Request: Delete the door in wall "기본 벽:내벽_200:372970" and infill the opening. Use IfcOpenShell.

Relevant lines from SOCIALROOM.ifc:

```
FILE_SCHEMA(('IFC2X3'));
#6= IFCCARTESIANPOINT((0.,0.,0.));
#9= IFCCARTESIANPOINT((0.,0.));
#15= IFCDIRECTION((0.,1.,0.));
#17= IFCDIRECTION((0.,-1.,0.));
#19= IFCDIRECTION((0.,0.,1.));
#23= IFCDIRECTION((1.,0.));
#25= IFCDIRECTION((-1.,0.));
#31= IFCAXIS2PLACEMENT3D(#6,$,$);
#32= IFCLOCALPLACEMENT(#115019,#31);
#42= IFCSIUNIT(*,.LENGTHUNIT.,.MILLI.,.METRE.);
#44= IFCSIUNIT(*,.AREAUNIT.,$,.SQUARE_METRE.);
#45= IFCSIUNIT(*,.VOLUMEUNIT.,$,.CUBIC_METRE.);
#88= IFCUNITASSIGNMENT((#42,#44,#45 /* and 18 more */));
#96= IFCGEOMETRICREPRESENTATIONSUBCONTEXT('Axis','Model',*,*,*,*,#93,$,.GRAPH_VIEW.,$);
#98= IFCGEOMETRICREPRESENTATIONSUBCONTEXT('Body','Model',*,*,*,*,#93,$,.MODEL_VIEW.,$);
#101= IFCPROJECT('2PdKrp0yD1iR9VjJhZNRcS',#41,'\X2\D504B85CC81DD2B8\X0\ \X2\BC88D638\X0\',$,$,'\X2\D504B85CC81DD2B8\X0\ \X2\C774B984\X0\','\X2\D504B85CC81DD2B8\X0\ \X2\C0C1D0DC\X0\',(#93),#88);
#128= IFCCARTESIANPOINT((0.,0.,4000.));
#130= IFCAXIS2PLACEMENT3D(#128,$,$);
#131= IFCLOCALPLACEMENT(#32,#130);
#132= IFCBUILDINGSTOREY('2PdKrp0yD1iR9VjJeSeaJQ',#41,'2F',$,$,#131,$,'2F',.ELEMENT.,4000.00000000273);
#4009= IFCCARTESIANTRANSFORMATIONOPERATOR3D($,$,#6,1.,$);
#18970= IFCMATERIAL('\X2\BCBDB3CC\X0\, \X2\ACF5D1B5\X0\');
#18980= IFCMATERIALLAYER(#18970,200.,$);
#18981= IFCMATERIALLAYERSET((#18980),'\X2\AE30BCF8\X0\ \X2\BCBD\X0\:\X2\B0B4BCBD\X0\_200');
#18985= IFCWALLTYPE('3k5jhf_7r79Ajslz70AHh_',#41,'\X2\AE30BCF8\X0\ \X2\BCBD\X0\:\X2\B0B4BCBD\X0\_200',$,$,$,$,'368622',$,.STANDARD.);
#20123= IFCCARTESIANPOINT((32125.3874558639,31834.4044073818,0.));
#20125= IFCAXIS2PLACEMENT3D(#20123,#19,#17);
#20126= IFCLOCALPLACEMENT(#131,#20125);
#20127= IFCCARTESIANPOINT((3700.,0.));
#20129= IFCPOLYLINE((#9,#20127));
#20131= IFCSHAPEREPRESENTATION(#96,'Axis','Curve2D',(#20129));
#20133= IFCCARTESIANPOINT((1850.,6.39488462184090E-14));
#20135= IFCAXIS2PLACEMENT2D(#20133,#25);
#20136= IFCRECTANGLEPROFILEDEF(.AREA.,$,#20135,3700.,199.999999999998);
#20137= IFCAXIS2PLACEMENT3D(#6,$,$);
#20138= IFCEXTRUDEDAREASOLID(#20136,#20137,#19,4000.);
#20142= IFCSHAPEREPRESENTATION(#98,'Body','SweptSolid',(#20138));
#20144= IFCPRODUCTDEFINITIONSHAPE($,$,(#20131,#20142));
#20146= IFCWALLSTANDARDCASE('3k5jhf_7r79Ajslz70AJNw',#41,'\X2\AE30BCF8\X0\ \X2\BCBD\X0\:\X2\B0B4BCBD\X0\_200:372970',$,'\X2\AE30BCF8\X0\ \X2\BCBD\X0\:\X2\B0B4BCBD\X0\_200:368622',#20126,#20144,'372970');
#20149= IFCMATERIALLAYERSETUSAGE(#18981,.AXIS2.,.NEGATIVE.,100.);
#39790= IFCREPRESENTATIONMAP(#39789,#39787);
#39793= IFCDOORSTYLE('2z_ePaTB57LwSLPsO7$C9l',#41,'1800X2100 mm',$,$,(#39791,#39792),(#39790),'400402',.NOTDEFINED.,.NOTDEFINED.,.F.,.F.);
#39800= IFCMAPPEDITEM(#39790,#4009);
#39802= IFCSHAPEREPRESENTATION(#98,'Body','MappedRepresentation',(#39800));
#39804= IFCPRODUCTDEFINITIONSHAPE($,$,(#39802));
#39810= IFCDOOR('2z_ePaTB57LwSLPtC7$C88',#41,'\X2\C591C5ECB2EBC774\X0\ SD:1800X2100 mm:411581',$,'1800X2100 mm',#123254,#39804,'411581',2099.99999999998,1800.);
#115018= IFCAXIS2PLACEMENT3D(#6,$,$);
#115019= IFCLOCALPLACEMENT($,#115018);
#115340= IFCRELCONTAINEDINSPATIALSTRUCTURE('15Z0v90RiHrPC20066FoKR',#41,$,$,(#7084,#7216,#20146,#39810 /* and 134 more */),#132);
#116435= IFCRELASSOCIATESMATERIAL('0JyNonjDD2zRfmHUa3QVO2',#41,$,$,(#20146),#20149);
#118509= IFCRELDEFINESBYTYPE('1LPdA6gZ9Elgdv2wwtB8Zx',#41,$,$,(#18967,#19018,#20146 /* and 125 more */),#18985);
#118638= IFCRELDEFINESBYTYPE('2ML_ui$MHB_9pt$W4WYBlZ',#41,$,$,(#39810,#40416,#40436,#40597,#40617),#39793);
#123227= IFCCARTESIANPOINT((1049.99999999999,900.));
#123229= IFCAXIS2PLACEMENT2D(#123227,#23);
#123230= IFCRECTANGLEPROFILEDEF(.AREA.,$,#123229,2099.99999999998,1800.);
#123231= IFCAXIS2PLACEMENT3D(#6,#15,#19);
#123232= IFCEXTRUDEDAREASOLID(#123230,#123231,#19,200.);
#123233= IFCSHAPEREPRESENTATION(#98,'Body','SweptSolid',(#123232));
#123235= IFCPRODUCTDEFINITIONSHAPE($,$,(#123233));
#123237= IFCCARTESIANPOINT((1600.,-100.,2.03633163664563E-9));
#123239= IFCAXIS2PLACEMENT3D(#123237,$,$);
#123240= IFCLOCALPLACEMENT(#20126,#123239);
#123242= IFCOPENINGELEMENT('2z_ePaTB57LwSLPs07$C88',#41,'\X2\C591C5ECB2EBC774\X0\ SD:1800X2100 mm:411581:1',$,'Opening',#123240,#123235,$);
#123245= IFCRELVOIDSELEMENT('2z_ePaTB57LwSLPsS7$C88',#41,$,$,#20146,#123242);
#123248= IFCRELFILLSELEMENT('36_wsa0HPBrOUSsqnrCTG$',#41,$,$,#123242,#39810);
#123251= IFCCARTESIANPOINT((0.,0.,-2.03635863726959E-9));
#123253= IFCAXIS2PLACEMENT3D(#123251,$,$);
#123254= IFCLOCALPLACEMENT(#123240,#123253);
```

```python
import ifcopenshell
import ifcopenshell.api.feature
import ifcopenshell.api.root
import ifcopenshell.geom
import ifcopenshell.util.shape

model = ifcopenshell.open("SOCIALROOM.ifc")
settings = ifcopenshell.geom.settings()


def volume(element):
    """Net volume in cubic metres, openings subtracted."""
    shape = ifcopenshell.geom.create_shape(settings, element)
    return ifcopenshell.util.shape.get_volume(shape.geometry)


door = model.by_id(39810)
opening = door.FillsVoids[0].RelatingOpeningElement
wall = opening.VoidsElements[0].RelatingBuildingElement
before = volume(wall)

ifcopenshell.api.root.remove_product(model, product=door)
ifcopenshell.api.feature.remove_feature(model, feature=opening)

after = volume(wall)

print(f"wall volume {before:.3f} -> {after:.3f} m3")

model.write("SOCIALROOM_updated.ifc")
```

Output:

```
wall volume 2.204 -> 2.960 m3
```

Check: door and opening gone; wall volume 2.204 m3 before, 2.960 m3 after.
